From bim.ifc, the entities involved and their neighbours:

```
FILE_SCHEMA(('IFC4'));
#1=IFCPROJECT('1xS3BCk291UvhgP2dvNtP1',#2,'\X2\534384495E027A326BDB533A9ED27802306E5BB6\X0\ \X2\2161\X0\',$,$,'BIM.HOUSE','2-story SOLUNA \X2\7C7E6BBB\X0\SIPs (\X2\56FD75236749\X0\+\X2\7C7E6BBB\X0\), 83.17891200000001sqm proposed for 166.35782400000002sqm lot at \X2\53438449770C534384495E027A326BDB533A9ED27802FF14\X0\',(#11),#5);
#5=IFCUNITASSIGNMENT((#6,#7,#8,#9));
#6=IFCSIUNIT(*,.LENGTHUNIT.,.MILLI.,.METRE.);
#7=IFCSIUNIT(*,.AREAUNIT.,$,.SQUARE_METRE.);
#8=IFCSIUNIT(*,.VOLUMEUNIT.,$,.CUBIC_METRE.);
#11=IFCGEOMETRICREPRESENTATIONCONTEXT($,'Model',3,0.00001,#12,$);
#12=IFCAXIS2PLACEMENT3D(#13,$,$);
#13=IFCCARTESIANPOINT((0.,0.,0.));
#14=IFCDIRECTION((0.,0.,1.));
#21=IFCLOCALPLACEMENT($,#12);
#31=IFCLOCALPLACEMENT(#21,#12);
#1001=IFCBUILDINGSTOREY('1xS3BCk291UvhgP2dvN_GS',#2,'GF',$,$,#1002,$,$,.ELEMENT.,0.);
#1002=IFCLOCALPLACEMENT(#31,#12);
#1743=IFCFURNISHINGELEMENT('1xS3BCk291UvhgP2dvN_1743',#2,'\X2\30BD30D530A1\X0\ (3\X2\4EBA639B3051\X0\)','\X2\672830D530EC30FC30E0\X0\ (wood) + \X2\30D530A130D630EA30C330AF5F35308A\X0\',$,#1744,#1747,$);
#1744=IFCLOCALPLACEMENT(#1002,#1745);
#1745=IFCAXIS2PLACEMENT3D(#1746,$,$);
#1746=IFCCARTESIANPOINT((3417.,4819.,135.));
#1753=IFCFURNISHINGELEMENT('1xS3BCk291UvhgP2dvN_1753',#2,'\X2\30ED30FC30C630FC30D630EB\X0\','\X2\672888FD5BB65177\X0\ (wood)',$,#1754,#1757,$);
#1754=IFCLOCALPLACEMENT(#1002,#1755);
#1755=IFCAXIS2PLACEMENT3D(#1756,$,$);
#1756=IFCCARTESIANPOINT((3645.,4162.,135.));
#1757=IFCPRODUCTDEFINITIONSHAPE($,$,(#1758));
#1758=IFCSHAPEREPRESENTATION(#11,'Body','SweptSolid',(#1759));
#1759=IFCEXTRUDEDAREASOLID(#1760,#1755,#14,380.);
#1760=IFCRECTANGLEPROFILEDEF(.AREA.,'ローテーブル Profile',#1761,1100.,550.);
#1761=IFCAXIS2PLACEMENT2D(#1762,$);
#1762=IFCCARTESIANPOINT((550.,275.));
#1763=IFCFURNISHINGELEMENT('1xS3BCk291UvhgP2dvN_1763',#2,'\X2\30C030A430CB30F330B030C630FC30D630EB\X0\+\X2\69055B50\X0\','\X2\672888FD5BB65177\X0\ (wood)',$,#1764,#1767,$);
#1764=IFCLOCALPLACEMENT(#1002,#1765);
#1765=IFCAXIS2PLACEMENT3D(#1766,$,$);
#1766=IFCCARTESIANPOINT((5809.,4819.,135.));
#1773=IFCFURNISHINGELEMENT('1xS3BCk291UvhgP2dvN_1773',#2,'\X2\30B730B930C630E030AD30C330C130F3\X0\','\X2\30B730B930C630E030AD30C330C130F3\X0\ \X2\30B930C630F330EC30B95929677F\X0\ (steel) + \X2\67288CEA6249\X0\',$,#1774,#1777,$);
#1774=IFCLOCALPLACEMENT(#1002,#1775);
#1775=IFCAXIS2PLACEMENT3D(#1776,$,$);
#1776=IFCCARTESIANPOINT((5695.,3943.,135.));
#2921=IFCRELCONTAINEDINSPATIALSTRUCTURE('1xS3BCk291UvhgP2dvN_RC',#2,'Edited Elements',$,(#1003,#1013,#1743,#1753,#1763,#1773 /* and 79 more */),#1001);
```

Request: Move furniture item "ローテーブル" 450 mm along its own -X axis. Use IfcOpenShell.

```python
import ifcopenshell
import ifcopenshell.api.geometry
import ifcopenshell.util.placement

model = ifcopenshell.open("bim.ifc")

item = model.by_guid("1xS3BCk291UvhgP2dvN_1753")
matrix = ifcopenshell.util.placement.get_local_placement(item.ObjectPlacement)
matrix[:3, 3] -= matrix[:3, 0] * 450.0
ifcopenshell.api.geometry.edit_object_placement(model, product=item, matrix=matrix, is_si=False)

print(ifcopenshell.util.placement.get_local_placement(item.ObjectPlacement).round(3) + 0.0)

model.write("bim_updated.ifc")
```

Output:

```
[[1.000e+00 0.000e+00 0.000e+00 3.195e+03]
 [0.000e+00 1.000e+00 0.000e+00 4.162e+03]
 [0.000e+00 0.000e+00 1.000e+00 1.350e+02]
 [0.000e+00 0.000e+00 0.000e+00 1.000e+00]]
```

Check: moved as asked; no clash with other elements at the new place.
